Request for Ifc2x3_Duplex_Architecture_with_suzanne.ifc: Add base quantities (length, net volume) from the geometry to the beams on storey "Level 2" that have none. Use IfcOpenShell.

First a look at what the model holds.

```python
import ifcopenshell
import ifcopenshell.util.element
import ifcopenshell.util.unit

model = ifcopenshell.open("Ifc2x3_Duplex_Architecture_with_suzanne.ifc")
print(model.schema)
for unit_type in ("LENGTHUNIT", "AREAUNIT", "VOLUMEUNIT"):
    print(unit_type, ifcopenshell.util.unit.calculate_unit_scale(model, unit_type))
storey = next(s for s in model.by_type("IfcBuildingStorey") if s.Name == "Level 2")
beams = [e for e in ifcopenshell.util.element.get_decomposition(storey) if e.is_a("IfcBeam")]
for e in sorted(beams, key=lambda e: e.id()):
    print(e.id(), e.is_a(), e.Name, list(ifcopenshell.util.element.get_psets(e, qtos_only=True)), sep=" | ")
```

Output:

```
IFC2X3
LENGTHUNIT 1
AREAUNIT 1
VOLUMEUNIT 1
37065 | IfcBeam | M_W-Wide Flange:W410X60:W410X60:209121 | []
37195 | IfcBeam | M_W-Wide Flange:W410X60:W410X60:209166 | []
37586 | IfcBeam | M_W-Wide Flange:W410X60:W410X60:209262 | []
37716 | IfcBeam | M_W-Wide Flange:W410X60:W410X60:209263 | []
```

```python
import ifcopenshell
import ifcopenshell.api.pset
import ifcopenshell.geom
import ifcopenshell.util.element
import ifcopenshell.util.shape
import ifcopenshell.util.unit

model = ifcopenshell.open("Ifc2x3_Duplex_Architecture_with_suzanne.ifc")
unit_scale = ifcopenshell.util.unit.calculate_unit_scale(model)
volume_scale = ifcopenshell.util.unit.calculate_unit_scale(model, "VOLUMEUNIT")
settings = ifcopenshell.geom.settings()

storey = next(s for s in model.by_type("IfcBuildingStorey") if s.Name == "Level 2")
beams = [e for e in ifcopenshell.util.element.get_decomposition(storey) if e.is_a("IfcBeam")]

for e in sorted(beams, key=lambda e: e.id()):
    if ifcopenshell.util.element.get_psets(e, qtos_only=True, should_inherit=False):
        continue
    # Geometry comes back in metres, in the element's own axes.
    shape = ifcopenshell.geom.create_shape(settings, e)
    values = {
        "Length": ifcopenshell.util.shape.get_max_xyz(shape.geometry) / unit_scale,
        "NetVolume": ifcopenshell.util.shape.get_volume(shape.geometry) / volume_scale,
    }
    qto = ifcopenshell.api.pset.add_qto(model, product=e, name="BaseQuantities")
    ifcopenshell.api.pset.edit_qto(model, qto=qto, properties=values)
    print(e.id(), {k: round(v, 3) for k, v in values.items()})

model.write("Ifc2x3_Duplex_Architecture_with_suzanne_edited.ifc")
```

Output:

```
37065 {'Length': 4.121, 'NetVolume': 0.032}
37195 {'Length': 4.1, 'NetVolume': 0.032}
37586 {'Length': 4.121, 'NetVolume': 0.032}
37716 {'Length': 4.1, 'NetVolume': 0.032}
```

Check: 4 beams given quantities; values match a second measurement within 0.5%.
